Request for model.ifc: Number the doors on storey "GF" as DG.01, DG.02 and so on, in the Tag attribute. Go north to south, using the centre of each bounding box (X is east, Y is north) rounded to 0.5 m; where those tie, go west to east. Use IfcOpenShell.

First a look at what the model holds.

```python
import ifcopenshell
import ifcopenshell.util.element
import ifcopenshell.util.placement

model = ifcopenshell.open("model.ifc")
print(model.schema)
storey = next(s for s in model.by_type("IfcBuildingStorey") if s.Name == "GF")
doors = [e for e in ifcopenshell.util.element.get_decomposition(storey) if e.is_a("IfcDoor")]
for e in sorted(doors, key=lambda e: e.id()):
    origin = ifcopenshell.util.placement.get_local_placement(e.ObjectPlacement)[:3, 3]
    print(e.id(), e.Tag, e.Name, origin.round(2) + 0.0, sep=" | ")
```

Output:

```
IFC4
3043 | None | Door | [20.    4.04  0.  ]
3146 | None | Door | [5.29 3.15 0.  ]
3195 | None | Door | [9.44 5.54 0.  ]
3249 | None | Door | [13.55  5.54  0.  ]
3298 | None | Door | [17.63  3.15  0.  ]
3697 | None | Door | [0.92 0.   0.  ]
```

```python
import ifcopenshell
import ifcopenshell.geom
import ifcopenshell.util.element
import ifcopenshell.util.shape

model = ifcopenshell.open("model.ifc")
settings = ifcopenshell.geom.settings()
settings.set("use-world-coords", True)


def centre(element):
    shape = ifcopenshell.geom.create_shape(settings, element)
    return ifcopenshell.util.shape.get_bbox_centroid(shape.geometry)


storey = next(s for s in model.by_type("IfcBuildingStorey") if s.Name == "GF")
doors = [e for e in ifcopenshell.util.element.get_decomposition(storey) if e.is_a("IfcDoor")]

# Insertion points can sit at a corner or the storey origin, so sort by the geometry (in metres).
centres = {e: centre(e) for e in doors}
doors.sort(key=lambda e: (-round(centres[e][1] / 0.5), centres[e][0]))

for i, e in enumerate(doors, start=1):
    number = f"DG.{i:02d}"
    e.Tag = number
    print(e.id(), number)

model.write("model_rev.ifc")
```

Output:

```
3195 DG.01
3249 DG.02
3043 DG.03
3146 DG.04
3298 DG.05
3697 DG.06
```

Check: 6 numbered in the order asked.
